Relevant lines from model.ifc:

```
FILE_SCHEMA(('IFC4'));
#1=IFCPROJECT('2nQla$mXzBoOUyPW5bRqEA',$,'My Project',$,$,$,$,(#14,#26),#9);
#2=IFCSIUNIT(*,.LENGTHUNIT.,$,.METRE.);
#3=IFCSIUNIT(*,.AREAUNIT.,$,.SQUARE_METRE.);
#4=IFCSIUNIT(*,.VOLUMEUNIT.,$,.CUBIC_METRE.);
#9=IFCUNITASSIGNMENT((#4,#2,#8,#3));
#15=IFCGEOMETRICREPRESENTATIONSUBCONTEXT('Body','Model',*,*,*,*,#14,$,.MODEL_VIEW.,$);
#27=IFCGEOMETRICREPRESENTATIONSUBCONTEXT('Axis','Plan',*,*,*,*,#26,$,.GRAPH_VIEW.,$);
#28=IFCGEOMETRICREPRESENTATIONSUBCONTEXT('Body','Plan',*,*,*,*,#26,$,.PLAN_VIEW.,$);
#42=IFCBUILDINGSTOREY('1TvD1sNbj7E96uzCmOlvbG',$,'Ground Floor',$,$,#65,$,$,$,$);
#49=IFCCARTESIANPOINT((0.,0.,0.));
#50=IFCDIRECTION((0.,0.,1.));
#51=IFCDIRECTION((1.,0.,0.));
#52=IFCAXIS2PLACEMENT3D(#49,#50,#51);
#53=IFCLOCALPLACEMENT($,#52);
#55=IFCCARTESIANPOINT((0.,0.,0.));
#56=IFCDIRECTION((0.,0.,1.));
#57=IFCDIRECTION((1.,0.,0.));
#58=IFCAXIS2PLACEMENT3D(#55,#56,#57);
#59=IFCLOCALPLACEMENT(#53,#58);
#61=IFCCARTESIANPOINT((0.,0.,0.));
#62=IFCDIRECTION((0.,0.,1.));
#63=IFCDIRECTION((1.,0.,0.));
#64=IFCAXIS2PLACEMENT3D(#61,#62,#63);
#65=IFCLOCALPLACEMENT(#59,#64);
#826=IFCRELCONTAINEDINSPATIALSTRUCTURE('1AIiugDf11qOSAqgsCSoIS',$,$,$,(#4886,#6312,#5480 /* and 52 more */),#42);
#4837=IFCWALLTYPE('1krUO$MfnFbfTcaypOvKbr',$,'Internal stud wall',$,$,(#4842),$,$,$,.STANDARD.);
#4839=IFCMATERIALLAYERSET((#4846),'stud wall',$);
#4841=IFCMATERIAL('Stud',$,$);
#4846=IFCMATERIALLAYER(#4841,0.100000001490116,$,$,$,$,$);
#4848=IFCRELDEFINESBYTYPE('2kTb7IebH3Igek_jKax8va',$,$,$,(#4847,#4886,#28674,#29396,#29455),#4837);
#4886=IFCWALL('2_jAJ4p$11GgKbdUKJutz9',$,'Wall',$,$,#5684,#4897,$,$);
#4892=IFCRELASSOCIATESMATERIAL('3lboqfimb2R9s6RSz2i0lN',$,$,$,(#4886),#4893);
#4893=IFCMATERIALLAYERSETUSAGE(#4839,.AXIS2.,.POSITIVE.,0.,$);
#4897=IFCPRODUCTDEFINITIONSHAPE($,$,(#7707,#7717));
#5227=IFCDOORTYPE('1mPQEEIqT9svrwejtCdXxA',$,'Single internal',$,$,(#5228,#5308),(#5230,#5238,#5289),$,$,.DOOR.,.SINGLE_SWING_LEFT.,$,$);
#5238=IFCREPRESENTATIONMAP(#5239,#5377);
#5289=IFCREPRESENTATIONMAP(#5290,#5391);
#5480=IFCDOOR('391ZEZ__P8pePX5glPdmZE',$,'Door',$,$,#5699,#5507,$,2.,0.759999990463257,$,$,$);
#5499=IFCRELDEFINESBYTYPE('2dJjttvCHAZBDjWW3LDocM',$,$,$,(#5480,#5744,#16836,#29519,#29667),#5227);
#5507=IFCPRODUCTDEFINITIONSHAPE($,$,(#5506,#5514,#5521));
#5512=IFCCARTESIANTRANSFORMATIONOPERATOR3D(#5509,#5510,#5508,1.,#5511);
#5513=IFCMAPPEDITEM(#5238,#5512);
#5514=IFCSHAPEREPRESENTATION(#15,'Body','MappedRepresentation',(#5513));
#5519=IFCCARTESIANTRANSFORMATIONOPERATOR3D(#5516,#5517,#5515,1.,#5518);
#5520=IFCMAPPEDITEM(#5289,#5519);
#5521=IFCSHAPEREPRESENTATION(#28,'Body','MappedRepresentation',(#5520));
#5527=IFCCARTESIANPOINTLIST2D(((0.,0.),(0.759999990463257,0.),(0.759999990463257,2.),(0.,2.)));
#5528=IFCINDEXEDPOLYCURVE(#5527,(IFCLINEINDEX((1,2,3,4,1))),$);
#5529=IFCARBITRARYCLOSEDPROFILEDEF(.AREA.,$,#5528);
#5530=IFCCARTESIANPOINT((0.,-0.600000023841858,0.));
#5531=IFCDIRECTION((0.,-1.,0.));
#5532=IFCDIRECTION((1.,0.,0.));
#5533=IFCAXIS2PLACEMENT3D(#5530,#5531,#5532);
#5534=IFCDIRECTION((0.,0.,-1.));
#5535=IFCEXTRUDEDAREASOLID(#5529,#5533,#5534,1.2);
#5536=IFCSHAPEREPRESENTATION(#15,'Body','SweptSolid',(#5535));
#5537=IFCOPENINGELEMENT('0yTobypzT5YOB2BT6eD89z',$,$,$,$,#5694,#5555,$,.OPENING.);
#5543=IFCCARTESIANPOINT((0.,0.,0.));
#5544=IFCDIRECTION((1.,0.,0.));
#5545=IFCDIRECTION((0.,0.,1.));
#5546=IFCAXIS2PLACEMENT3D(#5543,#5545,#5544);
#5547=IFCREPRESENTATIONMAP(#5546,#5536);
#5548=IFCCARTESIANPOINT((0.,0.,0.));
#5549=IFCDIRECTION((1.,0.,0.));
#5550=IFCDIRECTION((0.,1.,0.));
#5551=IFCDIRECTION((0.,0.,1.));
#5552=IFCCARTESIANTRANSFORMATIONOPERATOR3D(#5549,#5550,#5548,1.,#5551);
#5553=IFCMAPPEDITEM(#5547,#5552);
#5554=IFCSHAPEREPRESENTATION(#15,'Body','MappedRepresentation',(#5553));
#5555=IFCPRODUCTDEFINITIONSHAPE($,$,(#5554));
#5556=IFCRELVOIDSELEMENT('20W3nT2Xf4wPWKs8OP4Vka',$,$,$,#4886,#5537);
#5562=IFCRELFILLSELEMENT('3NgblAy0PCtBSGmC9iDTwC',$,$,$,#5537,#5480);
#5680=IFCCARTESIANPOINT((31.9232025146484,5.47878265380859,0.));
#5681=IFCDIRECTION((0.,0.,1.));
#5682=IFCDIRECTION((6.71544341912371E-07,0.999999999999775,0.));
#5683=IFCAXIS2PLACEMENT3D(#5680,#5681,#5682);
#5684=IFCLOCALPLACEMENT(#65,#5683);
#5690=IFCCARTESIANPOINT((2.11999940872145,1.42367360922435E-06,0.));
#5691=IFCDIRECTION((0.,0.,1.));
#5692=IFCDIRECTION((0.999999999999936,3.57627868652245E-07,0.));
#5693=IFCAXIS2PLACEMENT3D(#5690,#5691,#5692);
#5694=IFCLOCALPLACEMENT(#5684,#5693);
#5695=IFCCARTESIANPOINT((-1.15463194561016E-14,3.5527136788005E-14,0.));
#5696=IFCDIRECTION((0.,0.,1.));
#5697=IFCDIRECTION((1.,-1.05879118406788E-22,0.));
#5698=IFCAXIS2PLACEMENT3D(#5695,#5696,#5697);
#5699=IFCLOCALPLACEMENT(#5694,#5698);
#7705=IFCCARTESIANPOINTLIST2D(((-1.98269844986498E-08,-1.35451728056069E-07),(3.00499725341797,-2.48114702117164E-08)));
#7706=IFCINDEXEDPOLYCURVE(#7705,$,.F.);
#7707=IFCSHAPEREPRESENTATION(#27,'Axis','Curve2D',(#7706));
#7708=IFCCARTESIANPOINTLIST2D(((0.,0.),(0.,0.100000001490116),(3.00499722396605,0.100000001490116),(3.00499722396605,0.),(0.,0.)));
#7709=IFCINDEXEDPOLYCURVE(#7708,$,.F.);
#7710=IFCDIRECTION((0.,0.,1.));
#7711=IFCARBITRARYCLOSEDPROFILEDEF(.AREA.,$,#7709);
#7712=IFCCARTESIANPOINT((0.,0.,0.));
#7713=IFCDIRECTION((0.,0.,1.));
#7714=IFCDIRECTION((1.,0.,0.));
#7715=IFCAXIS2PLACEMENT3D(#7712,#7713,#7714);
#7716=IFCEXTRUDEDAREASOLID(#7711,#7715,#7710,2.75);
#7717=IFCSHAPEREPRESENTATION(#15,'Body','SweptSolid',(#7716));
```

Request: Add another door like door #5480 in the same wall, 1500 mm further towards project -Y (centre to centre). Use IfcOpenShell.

```python
import ifcopenshell
import ifcopenshell.api.feature
import ifcopenshell.api.geometry
import ifcopenshell.api.root
import ifcopenshell.geom
import ifcopenshell.util.element
import ifcopenshell.util.placement
import ifcopenshell.util.shape

model = ifcopenshell.open("model.ifc")
settings = ifcopenshell.geom.settings()


def volume(element):
    """Net volume in cubic metres, openings subtracted."""
    shape = ifcopenshell.geom.create_shape(settings, element)
    return ifcopenshell.util.shape.get_volume(shape.geometry)


door = model.by_id(5480)
opening = door.FillsVoids[0].RelatingOpeningElement
wall = opening.VoidsElements[0].RelatingBuildingElement
before = volume(wall)
shift = ifcopenshell.util.placement.get_local_placement(wall.ObjectPlacement)[:3, 0] * -1.5

# copy_class copies the void relationship, type, container and properties, but no geometry.
new_opening = ifcopenshell.api.root.copy_class(model, product=opening)
new_opening.Representation = ifcopenshell.util.element.copy_deep(
    model, opening.Representation, exclude=["IfcGeometricRepresentationContext", "IfcRepresentationMap"]
)
new_door = ifcopenshell.api.root.copy_class(model, product=door)
new_door.Representation = ifcopenshell.util.element.copy_deep(
    model, door.Representation, exclude=["IfcGeometricRepresentationContext", "IfcRepresentationMap"]
)
ifcopenshell.api.feature.add_filling(model, opening=new_opening, element=new_door)

for old, new in ((opening, new_opening), (door, new_door)):
    matrix = ifcopenshell.util.placement.get_local_placement(old.ObjectPlacement)
    matrix[:3, 3] += shift
    ifcopenshell.api.geometry.edit_object_placement(model, product=new, matrix=matrix, is_si=False)

after = volume(wall)

print(f"wall volume {before:.3f} -> {after:.3f} m3")

model.write("model_v2.ifc")
```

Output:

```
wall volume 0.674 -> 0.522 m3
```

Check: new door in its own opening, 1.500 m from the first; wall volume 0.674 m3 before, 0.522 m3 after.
